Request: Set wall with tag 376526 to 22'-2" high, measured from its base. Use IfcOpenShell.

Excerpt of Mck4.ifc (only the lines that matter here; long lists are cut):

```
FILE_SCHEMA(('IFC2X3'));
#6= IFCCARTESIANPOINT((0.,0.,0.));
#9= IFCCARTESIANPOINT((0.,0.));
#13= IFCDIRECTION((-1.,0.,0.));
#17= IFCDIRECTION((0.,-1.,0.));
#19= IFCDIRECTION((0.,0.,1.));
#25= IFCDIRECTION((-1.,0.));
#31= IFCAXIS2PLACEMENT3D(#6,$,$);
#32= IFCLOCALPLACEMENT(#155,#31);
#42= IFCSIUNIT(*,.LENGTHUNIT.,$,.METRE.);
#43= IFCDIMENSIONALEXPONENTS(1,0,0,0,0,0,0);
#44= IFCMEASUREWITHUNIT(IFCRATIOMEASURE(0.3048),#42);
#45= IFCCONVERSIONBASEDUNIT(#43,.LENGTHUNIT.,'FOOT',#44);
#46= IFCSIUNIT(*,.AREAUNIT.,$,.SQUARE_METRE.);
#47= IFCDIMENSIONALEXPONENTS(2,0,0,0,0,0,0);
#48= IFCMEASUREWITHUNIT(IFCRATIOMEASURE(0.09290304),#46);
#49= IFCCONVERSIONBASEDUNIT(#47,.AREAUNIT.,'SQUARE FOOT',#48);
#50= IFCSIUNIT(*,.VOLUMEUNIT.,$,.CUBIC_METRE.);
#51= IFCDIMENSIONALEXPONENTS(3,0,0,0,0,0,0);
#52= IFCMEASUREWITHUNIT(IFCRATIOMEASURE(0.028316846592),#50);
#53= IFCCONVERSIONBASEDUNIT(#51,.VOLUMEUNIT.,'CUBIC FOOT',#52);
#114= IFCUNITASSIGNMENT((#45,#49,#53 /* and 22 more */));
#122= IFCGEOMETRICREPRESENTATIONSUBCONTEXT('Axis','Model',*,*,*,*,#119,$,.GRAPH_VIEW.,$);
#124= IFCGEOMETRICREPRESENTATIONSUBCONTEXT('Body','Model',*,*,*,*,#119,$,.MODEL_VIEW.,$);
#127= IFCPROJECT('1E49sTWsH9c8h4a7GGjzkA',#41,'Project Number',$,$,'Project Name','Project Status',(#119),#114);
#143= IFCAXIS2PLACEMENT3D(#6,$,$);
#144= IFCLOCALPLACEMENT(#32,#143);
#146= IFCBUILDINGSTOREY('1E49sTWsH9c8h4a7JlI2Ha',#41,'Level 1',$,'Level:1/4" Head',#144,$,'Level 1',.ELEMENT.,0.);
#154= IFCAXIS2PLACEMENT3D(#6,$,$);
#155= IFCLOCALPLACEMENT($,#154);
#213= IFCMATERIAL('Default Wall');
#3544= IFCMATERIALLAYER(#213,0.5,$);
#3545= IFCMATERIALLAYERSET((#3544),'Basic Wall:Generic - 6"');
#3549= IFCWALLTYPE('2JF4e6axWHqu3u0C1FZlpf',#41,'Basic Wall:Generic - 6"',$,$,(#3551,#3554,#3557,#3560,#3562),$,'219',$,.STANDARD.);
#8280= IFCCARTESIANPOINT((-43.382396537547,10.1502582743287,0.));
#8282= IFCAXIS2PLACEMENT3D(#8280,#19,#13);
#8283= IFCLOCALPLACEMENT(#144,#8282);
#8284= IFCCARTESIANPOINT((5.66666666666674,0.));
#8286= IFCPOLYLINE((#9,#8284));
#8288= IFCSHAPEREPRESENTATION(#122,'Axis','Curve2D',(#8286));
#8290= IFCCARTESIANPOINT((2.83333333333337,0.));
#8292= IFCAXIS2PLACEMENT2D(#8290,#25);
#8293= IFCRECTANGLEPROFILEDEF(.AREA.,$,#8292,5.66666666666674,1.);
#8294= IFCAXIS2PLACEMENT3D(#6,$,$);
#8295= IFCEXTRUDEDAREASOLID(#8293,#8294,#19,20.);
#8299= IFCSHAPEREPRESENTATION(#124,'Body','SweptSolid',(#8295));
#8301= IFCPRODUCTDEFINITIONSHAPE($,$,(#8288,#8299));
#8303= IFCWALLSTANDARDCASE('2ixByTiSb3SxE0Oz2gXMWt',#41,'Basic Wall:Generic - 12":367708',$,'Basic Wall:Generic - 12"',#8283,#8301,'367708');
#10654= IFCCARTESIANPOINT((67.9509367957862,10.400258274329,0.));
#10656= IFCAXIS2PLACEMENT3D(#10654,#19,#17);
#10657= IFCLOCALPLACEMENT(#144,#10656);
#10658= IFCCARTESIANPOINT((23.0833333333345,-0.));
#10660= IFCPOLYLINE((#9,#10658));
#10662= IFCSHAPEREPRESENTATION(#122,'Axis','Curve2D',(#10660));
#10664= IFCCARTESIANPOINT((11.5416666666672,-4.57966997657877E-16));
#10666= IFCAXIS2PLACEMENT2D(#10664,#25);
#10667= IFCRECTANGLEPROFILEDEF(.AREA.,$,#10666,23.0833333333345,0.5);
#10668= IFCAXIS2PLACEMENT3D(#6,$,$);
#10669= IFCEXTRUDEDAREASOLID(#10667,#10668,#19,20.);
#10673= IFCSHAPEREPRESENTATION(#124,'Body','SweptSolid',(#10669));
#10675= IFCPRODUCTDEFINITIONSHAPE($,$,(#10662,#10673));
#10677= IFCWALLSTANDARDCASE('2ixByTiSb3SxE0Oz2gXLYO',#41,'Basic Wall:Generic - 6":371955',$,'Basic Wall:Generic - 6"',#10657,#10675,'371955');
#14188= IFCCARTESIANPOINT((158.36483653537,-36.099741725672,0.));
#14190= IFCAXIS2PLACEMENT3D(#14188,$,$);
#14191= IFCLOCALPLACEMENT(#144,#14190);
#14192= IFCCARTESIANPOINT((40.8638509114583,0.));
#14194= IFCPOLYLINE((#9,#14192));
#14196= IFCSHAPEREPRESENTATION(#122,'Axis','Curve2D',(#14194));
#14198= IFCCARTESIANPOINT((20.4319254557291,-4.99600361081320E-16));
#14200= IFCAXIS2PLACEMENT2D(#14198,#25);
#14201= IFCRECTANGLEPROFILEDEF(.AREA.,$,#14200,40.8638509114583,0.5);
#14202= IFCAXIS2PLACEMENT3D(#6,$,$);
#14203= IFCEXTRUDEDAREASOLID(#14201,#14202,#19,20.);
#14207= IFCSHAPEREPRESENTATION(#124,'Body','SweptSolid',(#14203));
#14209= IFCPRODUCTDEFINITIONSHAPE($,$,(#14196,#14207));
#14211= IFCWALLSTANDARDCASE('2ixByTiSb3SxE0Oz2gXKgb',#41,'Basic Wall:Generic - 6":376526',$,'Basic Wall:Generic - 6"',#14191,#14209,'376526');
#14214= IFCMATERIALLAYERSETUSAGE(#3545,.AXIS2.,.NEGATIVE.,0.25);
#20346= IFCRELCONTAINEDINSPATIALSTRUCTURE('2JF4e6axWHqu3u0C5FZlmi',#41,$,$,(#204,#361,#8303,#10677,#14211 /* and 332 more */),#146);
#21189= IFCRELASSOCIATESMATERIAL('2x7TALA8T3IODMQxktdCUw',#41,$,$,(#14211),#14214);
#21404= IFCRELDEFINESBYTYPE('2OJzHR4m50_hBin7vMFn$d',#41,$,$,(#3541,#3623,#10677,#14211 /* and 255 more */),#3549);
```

```python
import ifcopenshell
import ifcopenshell.geom
import ifcopenshell.util.representation
import ifcopenshell.util.shape
import ifcopenshell.util.unit

model = ifcopenshell.open("Mck4.ifc")
unit_scale = ifcopenshell.util.unit.calculate_unit_scale(model)
settings = ifcopenshell.geom.settings()


def volume(element):
    """Net volume in cubic metres, openings subtracted."""
    shape = ifcopenshell.geom.create_shape(settings, element)
    return ifcopenshell.util.shape.get_volume(shape.geometry)


wall = model.by_guid("2ixByTiSb3SxE0Oz2gXKgb")
before = volume(wall)

body = ifcopenshell.util.representation.get_representation(wall, "Model", "Body")
solid = body.Items[0]
old_height = solid.Depth
solid.Depth = 266 * 0.0254 / unit_scale
after = volume(wall)

print(f"height {old_height:g} -> {solid.Depth:g}, volume {before:.3f} -> {after:.3f} m3")

model.write("Mck4-out.ifc")
```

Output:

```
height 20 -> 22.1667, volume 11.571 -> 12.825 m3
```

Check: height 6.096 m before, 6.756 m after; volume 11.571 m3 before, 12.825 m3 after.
